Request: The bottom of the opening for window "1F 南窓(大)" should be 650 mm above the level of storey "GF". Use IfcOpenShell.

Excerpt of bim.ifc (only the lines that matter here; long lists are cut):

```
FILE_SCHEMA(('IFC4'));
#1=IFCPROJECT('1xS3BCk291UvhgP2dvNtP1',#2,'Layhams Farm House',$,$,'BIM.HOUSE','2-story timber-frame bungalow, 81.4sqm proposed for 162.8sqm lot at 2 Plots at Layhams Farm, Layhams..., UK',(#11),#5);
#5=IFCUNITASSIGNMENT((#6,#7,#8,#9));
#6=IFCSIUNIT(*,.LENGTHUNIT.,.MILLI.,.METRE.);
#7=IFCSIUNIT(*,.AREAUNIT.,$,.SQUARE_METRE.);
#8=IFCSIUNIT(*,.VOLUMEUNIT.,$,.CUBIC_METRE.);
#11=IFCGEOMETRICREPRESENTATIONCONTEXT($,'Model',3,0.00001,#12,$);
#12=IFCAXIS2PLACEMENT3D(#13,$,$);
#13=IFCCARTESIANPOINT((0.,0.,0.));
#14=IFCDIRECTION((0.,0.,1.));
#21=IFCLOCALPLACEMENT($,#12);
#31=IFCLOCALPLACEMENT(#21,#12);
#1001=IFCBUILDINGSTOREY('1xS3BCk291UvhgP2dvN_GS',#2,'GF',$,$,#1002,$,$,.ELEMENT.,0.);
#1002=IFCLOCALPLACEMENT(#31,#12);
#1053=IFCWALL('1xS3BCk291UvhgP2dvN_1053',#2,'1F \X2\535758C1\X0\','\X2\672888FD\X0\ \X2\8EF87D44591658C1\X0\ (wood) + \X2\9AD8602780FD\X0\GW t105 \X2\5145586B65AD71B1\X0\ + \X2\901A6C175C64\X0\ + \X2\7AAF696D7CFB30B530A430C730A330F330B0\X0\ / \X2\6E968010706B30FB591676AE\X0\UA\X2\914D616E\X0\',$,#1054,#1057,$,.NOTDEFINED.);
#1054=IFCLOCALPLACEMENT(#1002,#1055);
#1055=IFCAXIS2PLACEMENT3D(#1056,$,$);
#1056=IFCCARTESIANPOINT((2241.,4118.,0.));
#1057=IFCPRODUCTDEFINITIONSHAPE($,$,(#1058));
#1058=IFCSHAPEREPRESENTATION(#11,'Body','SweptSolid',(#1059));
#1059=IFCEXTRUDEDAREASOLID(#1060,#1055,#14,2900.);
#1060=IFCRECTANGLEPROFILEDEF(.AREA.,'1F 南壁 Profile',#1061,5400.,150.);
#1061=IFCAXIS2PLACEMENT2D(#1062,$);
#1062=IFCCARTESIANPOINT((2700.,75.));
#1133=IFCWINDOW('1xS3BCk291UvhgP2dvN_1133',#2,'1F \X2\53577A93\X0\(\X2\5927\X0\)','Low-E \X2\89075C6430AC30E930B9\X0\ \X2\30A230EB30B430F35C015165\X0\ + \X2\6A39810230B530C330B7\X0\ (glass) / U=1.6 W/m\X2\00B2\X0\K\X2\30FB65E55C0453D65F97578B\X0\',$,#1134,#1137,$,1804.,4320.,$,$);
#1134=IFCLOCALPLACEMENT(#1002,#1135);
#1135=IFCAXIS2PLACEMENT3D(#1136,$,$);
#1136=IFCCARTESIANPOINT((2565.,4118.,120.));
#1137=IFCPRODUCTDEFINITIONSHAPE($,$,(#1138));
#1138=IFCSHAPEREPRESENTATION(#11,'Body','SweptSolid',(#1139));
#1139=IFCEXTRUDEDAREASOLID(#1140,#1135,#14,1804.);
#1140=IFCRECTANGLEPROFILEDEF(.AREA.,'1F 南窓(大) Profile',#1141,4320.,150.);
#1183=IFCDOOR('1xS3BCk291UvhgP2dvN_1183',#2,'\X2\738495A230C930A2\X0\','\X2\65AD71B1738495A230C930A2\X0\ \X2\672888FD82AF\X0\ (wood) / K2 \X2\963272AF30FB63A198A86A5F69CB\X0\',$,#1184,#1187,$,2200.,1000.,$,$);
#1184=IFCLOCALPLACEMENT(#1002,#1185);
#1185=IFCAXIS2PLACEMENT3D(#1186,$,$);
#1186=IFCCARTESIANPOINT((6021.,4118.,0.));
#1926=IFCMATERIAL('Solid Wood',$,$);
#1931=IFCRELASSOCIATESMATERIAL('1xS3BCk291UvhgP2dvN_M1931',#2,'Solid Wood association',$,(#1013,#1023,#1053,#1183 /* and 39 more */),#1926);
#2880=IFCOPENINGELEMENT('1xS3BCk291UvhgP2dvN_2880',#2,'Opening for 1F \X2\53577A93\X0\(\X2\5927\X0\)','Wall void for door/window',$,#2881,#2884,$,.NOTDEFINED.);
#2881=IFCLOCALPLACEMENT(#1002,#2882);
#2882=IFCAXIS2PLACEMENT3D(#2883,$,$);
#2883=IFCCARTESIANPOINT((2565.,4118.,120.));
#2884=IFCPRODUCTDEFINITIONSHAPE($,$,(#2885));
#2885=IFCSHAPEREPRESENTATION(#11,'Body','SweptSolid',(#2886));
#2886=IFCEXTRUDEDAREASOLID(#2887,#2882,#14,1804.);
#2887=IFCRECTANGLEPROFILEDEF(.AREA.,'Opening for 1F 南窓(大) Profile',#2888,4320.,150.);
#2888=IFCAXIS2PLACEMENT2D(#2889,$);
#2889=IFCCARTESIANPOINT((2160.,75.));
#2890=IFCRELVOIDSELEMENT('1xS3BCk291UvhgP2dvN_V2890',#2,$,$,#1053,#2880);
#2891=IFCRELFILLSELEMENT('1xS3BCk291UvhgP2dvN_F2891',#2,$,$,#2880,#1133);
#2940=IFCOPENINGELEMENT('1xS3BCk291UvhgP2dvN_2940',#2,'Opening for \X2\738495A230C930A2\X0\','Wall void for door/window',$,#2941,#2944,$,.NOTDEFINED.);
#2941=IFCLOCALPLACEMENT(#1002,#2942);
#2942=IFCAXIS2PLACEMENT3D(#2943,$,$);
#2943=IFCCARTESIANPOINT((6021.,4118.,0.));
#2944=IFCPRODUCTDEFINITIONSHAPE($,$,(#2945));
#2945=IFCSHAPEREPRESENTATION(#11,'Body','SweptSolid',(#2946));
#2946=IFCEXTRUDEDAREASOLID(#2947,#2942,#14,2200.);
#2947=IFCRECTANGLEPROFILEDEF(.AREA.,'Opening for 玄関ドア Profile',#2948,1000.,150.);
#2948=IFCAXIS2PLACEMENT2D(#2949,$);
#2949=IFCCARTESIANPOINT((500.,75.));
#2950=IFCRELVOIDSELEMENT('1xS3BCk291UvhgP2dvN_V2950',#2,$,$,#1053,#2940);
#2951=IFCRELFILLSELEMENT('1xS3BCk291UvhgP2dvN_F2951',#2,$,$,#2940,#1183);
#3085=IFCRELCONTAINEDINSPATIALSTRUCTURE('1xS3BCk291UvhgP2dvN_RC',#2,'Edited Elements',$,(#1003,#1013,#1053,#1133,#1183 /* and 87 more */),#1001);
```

```python
import numpy as np
import ifcopenshell
import ifcopenshell.api.geometry
import ifcopenshell.geom
import ifcopenshell.util.element
import ifcopenshell.util.placement
import ifcopenshell.util.shape
import ifcopenshell.util.unit

model = ifcopenshell.open("bim.ifc")
unit_scale = ifcopenshell.util.unit.calculate_unit_scale(model)

window = model.by_id(1133)
opening = window.FillsVoids[0].RelatingOpeningElement
storey = ifcopenshell.util.element.get_container(window, ifc_class="IfcBuildingStorey")
level = ifcopenshell.util.placement.get_local_placement(storey.ObjectPlacement)[2, 3]

# The opening's origin need not be at the sill, so measure its lowest point.
shape = ifcopenshell.geom.create_shape(ifcopenshell.geom.settings(), opening)
bottom = ifcopenshell.util.shape.get_shape_bottom_elevation(shape, shape.geometry) / unit_scale
dz = level + 0.65 / unit_scale - bottom

shift = np.array([0.0, 0.0, dz])
# The window is not placed relative to its opening, so move both.
for product in (opening, window):
    matrix = ifcopenshell.util.placement.get_local_placement(product.ObjectPlacement)
    matrix[:3, 3] += shift
    ifcopenshell.api.geometry.edit_object_placement(model, product=product, matrix=matrix, is_si=False)

print(f"moved by {dz * unit_scale:+.3f} m")

model.write("bim-out.ifc")
```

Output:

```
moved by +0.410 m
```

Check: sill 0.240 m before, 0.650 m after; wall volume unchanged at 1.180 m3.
